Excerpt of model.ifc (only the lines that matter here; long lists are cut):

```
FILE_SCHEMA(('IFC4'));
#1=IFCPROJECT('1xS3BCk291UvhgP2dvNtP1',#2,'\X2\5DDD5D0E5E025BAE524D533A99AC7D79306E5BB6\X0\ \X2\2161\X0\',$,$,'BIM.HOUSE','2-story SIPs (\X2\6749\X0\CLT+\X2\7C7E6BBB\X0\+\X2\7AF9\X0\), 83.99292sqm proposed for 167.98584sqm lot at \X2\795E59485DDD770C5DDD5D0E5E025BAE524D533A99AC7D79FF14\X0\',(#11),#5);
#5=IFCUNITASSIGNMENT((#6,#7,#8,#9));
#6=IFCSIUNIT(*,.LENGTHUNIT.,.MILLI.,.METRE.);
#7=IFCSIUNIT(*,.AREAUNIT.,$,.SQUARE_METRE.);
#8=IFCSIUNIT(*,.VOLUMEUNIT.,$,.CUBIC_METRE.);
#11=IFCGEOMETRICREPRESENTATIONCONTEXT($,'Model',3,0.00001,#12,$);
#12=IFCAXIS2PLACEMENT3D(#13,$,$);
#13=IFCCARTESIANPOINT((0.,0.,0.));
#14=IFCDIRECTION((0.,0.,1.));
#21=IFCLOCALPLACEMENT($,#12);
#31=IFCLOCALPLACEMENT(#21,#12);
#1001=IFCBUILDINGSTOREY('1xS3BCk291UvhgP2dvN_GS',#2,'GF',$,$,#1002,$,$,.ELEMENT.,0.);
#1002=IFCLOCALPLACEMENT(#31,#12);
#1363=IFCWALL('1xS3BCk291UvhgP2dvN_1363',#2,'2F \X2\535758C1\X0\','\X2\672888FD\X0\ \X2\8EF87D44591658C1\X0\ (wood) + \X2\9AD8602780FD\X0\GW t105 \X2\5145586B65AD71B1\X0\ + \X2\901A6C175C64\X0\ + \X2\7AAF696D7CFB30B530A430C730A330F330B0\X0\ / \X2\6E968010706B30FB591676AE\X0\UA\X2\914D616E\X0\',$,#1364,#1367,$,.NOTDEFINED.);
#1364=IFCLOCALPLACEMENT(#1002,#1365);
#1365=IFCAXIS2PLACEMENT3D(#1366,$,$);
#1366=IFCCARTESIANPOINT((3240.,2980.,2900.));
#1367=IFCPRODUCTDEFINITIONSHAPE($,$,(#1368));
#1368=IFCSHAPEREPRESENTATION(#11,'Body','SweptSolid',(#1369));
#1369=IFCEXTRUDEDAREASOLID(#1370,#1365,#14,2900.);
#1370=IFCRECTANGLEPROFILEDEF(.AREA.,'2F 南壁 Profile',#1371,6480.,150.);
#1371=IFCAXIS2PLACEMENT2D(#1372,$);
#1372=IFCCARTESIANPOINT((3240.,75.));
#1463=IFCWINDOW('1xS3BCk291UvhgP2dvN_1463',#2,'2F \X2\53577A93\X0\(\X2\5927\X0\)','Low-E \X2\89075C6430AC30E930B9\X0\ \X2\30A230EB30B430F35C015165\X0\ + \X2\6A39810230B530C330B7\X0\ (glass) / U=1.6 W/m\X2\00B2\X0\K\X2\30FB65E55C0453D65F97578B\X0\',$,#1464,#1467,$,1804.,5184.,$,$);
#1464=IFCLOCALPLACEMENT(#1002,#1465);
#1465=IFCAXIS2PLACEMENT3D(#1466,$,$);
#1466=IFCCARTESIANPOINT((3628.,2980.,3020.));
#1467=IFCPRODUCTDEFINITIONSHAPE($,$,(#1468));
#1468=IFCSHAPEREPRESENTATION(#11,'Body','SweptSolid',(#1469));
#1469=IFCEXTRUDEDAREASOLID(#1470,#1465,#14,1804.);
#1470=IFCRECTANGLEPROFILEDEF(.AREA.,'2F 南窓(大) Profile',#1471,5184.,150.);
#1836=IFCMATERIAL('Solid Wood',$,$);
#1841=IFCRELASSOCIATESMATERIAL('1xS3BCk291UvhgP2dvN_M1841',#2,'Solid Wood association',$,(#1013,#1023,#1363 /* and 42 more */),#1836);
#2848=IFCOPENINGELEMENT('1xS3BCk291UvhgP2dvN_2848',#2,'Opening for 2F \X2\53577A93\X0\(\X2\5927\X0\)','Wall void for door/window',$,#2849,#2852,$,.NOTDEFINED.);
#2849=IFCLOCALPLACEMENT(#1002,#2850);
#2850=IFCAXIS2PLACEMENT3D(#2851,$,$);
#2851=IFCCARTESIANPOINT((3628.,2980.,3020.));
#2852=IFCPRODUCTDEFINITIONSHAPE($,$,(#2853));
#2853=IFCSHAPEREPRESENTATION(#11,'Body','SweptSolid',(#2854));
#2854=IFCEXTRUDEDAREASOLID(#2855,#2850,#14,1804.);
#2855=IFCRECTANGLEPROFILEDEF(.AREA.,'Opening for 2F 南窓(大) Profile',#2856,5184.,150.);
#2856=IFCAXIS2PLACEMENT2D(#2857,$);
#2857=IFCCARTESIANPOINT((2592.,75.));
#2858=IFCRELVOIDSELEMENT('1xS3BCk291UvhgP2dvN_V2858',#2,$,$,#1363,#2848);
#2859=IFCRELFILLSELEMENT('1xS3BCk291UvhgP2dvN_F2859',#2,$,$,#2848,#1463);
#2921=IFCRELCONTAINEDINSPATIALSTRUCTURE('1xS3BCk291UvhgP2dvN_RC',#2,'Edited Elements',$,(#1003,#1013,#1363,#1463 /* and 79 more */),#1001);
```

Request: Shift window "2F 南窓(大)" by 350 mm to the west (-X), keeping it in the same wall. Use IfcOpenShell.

```python
import ifcopenshell
import ifcopenshell.api.geometry
import ifcopenshell.util.placement

model = ifcopenshell.open("model.ifc")

window = model.by_guid("1xS3BCk291UvhgP2dvN_1463")
opening = window.FillsVoids[0].RelatingOpeningElement
wall = opening.VoidsElements[0].RelatingBuildingElement

wall_matrix = ifcopenshell.util.placement.get_local_placement(wall.ObjectPlacement)
shift = wall_matrix[:3, 0] * -350.0
before = ifcopenshell.util.placement.get_local_placement(window.ObjectPlacement)[:3, 3].copy()

# The window is not placed relative to its opening, so move both.
for product in (opening, window):
    matrix = ifcopenshell.util.placement.get_local_placement(product.ObjectPlacement)
    matrix[:3, 3] += shift
    ifcopenshell.api.geometry.edit_object_placement(model, product=product, matrix=matrix, is_si=False)

after = ifcopenshell.util.placement.get_local_placement(window.ObjectPlacement)[:3, 3]
print("window moved by", (after - before).round(3) + 0.0)

model.write("model-out.ifc")
```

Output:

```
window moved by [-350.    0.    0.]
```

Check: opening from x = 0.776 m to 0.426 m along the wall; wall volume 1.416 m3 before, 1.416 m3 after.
